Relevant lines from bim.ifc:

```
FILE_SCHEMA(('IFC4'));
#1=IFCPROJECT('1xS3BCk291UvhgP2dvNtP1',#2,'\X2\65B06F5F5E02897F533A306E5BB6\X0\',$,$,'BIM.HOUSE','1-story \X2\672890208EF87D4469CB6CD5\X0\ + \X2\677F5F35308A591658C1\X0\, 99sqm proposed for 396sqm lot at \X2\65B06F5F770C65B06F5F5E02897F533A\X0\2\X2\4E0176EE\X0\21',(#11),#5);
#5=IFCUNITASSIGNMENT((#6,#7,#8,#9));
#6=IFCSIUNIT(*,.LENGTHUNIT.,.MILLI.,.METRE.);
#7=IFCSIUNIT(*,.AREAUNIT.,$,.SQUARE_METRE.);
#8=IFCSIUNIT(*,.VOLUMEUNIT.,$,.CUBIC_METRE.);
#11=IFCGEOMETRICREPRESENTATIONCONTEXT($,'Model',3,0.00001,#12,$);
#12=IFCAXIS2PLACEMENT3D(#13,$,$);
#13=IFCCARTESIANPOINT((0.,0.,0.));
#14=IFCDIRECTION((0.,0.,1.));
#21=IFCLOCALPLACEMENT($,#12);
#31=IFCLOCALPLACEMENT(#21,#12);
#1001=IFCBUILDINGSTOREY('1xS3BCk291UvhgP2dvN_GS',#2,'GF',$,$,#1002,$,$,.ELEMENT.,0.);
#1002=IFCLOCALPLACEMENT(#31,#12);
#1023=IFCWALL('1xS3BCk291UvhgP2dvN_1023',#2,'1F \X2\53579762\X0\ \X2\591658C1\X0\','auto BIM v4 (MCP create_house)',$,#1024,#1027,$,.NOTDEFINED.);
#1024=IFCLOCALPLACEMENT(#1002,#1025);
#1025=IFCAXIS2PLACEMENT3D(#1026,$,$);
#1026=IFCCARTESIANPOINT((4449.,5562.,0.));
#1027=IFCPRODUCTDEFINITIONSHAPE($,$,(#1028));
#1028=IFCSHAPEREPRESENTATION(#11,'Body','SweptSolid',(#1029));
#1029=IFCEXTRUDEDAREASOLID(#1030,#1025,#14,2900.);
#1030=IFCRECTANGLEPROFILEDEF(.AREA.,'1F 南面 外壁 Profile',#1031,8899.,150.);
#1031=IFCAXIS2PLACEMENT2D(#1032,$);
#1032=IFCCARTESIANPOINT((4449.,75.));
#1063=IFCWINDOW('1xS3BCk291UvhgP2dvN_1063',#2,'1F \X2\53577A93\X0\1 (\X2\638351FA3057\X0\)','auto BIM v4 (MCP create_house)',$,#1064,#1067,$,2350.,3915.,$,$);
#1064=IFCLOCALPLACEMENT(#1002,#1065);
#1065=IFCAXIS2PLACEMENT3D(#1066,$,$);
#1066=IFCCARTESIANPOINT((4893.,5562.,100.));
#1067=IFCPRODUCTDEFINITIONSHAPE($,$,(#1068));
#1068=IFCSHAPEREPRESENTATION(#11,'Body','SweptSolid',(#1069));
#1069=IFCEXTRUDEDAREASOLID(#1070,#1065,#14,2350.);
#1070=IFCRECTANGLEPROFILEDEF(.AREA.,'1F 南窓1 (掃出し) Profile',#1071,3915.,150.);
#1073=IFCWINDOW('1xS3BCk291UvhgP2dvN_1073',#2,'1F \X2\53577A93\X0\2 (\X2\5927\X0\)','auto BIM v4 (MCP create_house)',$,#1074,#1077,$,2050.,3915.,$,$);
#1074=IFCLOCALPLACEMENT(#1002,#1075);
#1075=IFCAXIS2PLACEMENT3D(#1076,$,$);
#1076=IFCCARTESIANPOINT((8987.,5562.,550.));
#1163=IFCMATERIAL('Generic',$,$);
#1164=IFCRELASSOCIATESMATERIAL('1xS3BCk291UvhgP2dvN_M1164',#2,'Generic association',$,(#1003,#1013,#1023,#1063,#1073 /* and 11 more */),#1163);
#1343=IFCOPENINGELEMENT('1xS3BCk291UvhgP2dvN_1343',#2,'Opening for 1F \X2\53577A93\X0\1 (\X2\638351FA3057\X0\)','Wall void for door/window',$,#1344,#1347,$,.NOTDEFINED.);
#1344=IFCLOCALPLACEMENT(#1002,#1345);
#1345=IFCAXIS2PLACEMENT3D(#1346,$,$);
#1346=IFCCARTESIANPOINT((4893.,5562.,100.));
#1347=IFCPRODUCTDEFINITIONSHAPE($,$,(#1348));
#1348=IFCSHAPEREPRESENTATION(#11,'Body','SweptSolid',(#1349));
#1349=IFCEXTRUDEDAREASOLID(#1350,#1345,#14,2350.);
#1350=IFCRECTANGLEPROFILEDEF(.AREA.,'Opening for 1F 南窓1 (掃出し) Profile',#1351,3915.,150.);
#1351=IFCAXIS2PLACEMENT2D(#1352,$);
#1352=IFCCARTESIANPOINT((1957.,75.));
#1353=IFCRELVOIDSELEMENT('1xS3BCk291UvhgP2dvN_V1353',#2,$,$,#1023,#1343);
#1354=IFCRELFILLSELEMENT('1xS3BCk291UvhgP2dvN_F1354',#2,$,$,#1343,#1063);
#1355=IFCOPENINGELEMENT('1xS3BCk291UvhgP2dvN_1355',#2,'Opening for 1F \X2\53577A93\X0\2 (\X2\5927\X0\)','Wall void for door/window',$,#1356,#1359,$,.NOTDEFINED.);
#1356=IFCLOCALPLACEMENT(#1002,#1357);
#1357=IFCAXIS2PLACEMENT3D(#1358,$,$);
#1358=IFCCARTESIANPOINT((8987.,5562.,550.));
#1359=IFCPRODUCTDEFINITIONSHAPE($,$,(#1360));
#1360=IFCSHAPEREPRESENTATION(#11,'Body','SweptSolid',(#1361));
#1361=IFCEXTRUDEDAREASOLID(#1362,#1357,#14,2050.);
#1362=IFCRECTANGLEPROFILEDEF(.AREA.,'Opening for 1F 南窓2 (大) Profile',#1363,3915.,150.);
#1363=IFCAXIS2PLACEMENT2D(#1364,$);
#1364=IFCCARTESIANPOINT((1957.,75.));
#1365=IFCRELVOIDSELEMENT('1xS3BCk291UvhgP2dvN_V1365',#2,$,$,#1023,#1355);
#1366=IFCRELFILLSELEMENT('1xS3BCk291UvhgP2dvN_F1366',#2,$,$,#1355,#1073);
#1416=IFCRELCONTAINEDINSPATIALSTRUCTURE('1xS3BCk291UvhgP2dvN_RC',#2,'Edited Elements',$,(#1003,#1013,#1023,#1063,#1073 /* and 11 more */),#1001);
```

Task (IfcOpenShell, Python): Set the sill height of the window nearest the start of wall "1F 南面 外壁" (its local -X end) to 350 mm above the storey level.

```python
import numpy as np
import ifcopenshell
import ifcopenshell.api.geometry
import ifcopenshell.geom
import ifcopenshell.util.element
import ifcopenshell.util.placement
import ifcopenshell.util.shape
import ifcopenshell.util.unit

model = ifcopenshell.open("bim.ifc")
unit_scale = ifcopenshell.util.unit.calculate_unit_scale(model)

window = model.by_id(1063)
opening = window.FillsVoids[0].RelatingOpeningElement
storey = ifcopenshell.util.element.get_container(window, ifc_class="IfcBuildingStorey")
level = ifcopenshell.util.placement.get_local_placement(storey.ObjectPlacement)[2, 3]

# The opening's origin need not be at the sill, so measure its lowest point.
shape = ifcopenshell.geom.create_shape(ifcopenshell.geom.settings(), opening)
bottom = ifcopenshell.util.shape.get_shape_bottom_elevation(shape, shape.geometry) / unit_scale
dz = level + 350.0 - bottom

shift = np.array([0.0, 0.0, dz])
# The window is not placed relative to its opening, so move both.
for product in (opening, window):
    matrix = ifcopenshell.util.placement.get_local_placement(product.ObjectPlacement)
    matrix[:3, 3] += shift
    ifcopenshell.api.geometry.edit_object_placement(model, product=product, matrix=matrix, is_si=False)

print(f"moved by {dz * unit_scale:+.3f} m")

model.write("bim_updated.ifc")
```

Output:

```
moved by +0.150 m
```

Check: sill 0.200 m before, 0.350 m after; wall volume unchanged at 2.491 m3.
